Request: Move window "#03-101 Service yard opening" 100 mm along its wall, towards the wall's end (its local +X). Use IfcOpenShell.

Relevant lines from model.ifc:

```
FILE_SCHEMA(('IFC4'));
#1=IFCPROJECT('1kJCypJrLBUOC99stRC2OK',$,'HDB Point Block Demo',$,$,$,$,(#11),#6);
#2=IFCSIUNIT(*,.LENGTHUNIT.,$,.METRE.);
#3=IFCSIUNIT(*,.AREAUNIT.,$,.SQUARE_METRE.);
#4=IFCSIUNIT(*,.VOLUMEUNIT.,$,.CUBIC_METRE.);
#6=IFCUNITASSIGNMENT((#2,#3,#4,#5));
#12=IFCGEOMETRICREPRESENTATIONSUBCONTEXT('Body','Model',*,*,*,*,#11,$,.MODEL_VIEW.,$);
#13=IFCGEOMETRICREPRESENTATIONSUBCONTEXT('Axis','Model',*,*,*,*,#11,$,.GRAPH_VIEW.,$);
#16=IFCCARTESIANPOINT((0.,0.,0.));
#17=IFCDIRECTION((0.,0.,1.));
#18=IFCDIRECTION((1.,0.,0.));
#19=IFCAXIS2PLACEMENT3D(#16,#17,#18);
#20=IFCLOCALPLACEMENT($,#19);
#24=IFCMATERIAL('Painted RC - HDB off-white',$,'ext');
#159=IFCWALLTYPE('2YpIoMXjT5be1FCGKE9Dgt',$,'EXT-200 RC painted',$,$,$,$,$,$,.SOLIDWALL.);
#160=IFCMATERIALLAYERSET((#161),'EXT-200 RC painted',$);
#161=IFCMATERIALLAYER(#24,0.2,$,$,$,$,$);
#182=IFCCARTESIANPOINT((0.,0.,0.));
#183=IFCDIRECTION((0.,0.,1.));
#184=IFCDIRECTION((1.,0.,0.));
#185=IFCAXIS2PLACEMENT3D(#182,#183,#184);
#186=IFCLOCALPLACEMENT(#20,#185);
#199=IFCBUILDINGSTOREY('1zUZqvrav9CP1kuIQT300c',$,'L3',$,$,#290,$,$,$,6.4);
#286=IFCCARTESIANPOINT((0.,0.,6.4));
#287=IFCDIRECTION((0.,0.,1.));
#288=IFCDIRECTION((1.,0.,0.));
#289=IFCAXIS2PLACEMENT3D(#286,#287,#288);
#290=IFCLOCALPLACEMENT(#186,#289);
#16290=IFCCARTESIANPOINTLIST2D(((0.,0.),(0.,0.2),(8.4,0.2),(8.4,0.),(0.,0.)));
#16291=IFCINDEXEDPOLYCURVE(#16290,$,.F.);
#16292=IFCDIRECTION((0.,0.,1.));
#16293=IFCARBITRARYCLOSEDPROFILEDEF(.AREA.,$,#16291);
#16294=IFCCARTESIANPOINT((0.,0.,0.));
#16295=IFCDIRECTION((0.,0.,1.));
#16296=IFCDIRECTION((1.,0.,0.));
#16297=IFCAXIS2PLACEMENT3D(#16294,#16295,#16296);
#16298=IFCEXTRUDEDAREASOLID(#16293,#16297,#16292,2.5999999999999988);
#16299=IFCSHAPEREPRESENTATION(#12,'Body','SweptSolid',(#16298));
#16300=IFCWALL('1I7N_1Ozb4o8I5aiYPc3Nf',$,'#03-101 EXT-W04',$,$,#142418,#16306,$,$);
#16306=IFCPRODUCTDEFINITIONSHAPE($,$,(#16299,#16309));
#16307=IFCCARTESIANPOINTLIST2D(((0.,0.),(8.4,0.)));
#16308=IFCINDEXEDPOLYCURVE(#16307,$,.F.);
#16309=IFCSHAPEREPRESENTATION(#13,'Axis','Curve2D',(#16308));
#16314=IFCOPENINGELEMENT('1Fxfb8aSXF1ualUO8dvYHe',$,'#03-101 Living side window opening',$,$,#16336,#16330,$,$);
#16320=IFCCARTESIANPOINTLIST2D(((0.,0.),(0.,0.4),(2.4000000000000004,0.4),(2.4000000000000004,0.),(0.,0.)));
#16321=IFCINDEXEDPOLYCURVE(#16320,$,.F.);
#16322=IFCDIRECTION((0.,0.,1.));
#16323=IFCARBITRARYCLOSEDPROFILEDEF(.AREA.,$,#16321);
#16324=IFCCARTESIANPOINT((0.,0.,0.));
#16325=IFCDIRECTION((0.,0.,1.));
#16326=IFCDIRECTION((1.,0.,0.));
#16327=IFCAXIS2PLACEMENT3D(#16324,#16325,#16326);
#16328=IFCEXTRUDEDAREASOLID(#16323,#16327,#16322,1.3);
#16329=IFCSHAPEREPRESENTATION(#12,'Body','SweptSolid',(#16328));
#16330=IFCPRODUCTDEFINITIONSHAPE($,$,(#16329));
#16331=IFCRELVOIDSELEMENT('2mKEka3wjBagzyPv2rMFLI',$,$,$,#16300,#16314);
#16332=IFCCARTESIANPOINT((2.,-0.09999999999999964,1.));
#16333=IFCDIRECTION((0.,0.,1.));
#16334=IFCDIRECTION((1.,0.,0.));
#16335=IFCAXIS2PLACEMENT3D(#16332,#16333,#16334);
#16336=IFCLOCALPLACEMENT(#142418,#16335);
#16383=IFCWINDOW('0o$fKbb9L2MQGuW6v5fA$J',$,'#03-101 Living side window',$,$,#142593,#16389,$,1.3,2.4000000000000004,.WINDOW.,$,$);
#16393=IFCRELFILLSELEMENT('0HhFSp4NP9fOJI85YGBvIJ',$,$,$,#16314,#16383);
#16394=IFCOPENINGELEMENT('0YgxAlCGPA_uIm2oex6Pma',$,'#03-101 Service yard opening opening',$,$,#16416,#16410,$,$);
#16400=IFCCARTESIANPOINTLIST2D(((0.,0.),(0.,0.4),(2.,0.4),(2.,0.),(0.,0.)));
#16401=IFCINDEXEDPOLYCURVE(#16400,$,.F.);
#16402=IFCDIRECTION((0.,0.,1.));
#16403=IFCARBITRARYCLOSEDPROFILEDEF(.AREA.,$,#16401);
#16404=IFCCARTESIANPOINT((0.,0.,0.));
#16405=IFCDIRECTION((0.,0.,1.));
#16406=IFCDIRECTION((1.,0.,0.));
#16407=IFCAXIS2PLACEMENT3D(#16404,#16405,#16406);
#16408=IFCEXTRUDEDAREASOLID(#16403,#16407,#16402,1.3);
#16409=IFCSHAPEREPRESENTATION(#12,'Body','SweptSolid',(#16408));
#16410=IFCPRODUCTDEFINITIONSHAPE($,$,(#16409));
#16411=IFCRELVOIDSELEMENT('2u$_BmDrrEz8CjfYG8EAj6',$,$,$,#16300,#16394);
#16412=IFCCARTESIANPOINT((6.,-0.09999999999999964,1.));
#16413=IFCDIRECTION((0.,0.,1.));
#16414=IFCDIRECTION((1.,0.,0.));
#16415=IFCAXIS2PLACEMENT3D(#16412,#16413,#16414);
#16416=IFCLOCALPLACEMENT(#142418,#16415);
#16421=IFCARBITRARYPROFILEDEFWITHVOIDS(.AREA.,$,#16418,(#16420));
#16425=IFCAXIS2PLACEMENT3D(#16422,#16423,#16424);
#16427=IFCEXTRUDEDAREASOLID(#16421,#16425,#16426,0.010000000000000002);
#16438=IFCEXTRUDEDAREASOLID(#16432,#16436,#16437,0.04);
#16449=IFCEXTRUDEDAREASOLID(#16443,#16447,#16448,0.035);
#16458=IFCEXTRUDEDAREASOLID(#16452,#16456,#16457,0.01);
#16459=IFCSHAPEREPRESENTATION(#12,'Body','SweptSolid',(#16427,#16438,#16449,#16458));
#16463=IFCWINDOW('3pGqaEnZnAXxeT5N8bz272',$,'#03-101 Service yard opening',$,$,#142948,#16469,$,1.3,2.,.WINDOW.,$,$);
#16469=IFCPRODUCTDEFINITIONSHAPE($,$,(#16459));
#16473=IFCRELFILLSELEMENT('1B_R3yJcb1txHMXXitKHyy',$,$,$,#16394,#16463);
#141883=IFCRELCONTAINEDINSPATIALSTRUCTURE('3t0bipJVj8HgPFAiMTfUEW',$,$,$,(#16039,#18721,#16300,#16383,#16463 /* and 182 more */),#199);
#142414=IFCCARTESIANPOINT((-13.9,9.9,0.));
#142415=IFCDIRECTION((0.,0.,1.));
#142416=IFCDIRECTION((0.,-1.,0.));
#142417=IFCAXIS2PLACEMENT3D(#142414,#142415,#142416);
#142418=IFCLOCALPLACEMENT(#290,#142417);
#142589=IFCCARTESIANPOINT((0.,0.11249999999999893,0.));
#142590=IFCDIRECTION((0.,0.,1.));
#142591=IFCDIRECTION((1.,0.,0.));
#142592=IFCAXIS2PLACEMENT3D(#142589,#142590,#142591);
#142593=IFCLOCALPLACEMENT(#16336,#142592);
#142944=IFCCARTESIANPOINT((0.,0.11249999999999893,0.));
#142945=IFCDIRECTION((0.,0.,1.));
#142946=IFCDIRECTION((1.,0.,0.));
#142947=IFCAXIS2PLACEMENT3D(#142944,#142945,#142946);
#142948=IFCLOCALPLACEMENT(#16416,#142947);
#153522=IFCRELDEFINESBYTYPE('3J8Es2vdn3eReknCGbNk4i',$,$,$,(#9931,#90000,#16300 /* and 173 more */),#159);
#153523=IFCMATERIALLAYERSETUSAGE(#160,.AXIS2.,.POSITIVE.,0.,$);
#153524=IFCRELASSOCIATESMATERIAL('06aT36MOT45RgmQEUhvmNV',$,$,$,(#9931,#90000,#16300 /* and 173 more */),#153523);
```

```python
import ifcopenshell
import ifcopenshell.api.geometry
import ifcopenshell.util.placement
import ifcopenshell.util.unit

model = ifcopenshell.open("model.ifc")
unit_scale = ifcopenshell.util.unit.calculate_unit_scale(model)

window = model.by_guid("3pGqaEnZnAXxeT5N8bz272")
opening = window.FillsVoids[0].RelatingOpeningElement
wall = opening.VoidsElements[0].RelatingBuildingElement

wall_matrix = ifcopenshell.util.placement.get_local_placement(wall.ObjectPlacement)
shift = wall_matrix[:3, 0] * 0.1 / unit_scale
before = ifcopenshell.util.placement.get_local_placement(window.ObjectPlacement)[:3, 3].copy()

# The window is placed relative to its opening, so it follows when the opening moves.
matrix = ifcopenshell.util.placement.get_local_placement(opening.ObjectPlacement)
matrix[:3, 3] += shift
ifcopenshell.api.geometry.edit_object_placement(
    model, product=opening, matrix=matrix, is_si=False, should_transform_children=True
)

after = ifcopenshell.util.placement.get_local_placement(window.ObjectPlacement)[:3, 3]
print("window moved by", (after - before).round(3) + 0.0)

model.write("model_edited.ifc")
```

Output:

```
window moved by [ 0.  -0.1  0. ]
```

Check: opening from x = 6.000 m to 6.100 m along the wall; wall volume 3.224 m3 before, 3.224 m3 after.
